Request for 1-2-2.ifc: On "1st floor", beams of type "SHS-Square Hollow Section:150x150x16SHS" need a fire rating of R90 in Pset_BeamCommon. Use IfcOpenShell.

First a look at what the model holds.

```python
import ifcopenshell
import ifcopenshell.util.element

model = ifcopenshell.open("1-2-2.ifc")
print(model.schema)
storey = next(s for s in model.by_type("IfcBuildingStorey") if s.Name == "1st floor")
beams = [e for e in ifcopenshell.util.element.get_decomposition(storey) if e.is_a("IfcBeam")]
seen = {}
for e in beams:
    element_type = ifcopenshell.util.element.get_type(e)
    key = (element_type.Name if element_type != e and element_type else None, ifcopenshell.util.element.get_pset(e, "Pset_BeamCommon", "FireRating"))
    seen[key] = seen.get(key, 0) + 1
for (name, value), count in sorted(seen.items(), key=str):
    print(count, "x", name, "|", value)
```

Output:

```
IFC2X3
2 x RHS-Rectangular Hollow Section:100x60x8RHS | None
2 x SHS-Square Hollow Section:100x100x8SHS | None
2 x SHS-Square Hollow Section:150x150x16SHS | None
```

```python
import ifcopenshell
import ifcopenshell.api.pset
import ifcopenshell.util.element

model = ifcopenshell.open("1-2-2.ifc")

storey = next(s for s in model.by_type("IfcBuildingStorey") if s.Name == "1st floor")
beams = [e for e in ifcopenshell.util.element.get_decomposition(storey) if e.is_a("IfcBeam")]

count = 0
for e in beams:
    element_type = ifcopenshell.util.element.get_type(e)
    if element_type in (None, e) or element_type.Name != "SHS-Square Hollow Section:150x150x16SHS":
        continue
    # add_pset returns the element's existing set when there is one.
    pset = ifcopenshell.api.pset.add_pset(model, product=e, name="Pset_BeamCommon")
    ifcopenshell.api.pset.edit_pset(model, pset=pset, properties={"FireRating": "R90"})
    count += 1

print(count, "beams updated")

model.write("1-2-2-out.ifc")
```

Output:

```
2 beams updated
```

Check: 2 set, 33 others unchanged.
